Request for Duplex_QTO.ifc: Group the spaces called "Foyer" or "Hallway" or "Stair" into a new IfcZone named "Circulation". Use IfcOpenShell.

First a look at what the model holds.

```python
import ifcopenshell

model = ifcopenshell.open("Duplex_QTO.ifc")
print(model.schema)
seen = {}
for space in model.by_type("IfcSpace"):
    seen[space.LongName] = seen.get(space.LongName, 0) + 1
for name, count in sorted(seen.items(), key=str):
    print(count, "x", name)
print("zones:", [z.Name for z in model.by_type("IfcZone")][:20])
```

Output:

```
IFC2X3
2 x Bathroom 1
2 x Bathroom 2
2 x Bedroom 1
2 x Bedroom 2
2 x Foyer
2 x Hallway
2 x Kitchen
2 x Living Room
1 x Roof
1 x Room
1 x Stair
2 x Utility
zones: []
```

```python
import ifcopenshell
import ifcopenshell.api.group
import ifcopenshell.api.root

model = ifcopenshell.open("Duplex_QTO.ifc")

names = {"Foyer", "Hallway", "Stair"}
spaces = [s for s in model.by_type("IfcSpace") if s.LongName in names]

zone = ifcopenshell.api.root.create_entity(model, ifc_class="IfcZone", name="Circulation")
ifcopenshell.api.group.assign_group(model, products=spaces, group=zone)
print(len(spaces), "spaces in", zone.Name)

model.write("Duplex_QTO_v2.ifc")
```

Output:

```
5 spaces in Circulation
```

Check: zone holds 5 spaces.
